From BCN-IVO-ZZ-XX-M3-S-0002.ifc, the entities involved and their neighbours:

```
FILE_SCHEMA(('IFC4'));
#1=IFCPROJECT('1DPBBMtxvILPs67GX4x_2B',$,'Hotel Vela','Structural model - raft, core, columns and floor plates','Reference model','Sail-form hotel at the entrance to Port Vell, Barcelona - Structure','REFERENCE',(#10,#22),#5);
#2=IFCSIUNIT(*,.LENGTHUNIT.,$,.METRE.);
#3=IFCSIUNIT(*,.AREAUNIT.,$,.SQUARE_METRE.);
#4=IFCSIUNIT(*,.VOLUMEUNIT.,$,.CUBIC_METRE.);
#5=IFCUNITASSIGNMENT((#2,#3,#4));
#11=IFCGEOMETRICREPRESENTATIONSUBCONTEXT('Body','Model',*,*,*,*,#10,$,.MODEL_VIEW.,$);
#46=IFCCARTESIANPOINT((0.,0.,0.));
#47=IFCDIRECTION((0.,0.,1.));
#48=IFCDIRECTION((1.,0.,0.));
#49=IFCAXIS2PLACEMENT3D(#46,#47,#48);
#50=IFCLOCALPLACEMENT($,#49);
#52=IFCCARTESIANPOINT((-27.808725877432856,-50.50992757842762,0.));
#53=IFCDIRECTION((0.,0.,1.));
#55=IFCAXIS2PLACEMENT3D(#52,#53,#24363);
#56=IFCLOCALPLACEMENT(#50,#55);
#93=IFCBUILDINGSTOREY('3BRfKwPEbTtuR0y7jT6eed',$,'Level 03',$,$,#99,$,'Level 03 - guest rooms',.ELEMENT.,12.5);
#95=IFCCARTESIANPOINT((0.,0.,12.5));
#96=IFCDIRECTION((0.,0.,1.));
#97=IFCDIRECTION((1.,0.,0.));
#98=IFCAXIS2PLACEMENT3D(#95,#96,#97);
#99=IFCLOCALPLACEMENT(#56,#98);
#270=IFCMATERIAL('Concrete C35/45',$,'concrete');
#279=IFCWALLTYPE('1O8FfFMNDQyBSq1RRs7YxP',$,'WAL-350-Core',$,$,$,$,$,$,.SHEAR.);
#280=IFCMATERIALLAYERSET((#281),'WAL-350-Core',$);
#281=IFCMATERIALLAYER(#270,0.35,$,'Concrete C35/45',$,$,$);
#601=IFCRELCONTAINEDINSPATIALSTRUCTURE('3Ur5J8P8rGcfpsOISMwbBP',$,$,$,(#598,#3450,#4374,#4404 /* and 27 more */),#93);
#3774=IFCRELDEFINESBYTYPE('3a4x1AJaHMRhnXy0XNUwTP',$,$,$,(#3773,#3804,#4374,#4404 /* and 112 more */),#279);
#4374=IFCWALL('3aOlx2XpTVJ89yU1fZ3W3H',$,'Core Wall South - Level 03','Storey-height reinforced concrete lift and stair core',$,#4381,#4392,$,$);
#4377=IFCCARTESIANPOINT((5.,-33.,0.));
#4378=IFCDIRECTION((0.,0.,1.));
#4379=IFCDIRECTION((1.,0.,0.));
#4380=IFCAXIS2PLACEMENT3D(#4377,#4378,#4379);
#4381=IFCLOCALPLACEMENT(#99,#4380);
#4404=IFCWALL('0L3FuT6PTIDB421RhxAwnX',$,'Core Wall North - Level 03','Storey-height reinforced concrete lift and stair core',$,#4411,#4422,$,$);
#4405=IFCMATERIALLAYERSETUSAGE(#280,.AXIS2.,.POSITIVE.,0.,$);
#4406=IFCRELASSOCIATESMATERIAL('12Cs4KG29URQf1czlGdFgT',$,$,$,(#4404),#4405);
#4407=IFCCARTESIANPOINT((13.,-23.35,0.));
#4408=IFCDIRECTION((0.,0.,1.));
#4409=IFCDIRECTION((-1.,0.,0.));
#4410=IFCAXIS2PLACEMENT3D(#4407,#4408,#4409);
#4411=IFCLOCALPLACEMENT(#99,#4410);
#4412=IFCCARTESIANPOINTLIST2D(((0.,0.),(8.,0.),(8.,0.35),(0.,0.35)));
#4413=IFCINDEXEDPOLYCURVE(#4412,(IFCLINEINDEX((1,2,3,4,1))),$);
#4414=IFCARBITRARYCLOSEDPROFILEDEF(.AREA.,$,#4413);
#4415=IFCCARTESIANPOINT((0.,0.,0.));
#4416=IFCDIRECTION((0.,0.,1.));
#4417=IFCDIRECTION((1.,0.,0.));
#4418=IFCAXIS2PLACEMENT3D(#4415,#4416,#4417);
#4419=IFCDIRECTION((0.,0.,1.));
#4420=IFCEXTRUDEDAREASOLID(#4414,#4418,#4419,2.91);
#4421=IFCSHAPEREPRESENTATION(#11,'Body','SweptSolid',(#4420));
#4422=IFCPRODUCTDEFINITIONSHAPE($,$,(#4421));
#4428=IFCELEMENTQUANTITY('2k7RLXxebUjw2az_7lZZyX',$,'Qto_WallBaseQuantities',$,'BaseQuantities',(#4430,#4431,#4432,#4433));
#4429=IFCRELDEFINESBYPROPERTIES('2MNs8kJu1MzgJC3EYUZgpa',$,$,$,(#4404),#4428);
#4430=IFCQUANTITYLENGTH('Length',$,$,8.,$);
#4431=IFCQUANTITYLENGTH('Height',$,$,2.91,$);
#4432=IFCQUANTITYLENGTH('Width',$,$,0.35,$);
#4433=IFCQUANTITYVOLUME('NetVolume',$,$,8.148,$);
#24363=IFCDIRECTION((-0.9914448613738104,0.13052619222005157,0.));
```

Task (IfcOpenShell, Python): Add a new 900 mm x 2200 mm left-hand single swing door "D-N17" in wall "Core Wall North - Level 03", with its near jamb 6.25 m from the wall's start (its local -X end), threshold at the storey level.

```python
import numpy as np
import ifcopenshell
import ifcopenshell.api.feature
import ifcopenshell.api.geometry
import ifcopenshell.api.pset
import ifcopenshell.api.root
import ifcopenshell.api.spatial
import ifcopenshell.geom
import ifcopenshell.util.element
import ifcopenshell.util.placement
import ifcopenshell.util.representation
import ifcopenshell.util.shape
import ifcopenshell.util.unit

model = ifcopenshell.open("BCN-IVO-ZZ-XX-M3-S-0002.ifc")
unit_scale = ifcopenshell.util.unit.calculate_unit_scale(model)
volume_scale = ifcopenshell.util.unit.calculate_unit_scale(model, "VOLUMEUNIT")
settings = ifcopenshell.geom.settings()


def volume(element):
    """Net volume in cubic metres, openings subtracted."""
    shape = ifcopenshell.geom.create_shape(settings, element)
    return ifcopenshell.util.shape.get_volume(shape.geometry)


wall = model.by_id(4404)
storey = ifcopenshell.util.element.get_container(wall, ifc_class="IfcBuildingStorey")
context = ifcopenshell.util.representation.get_context(model, "Model", "Body", "MODEL_VIEW")
before = volume(wall)

width, height, from_end, sill = 0.9, 2.2, 6.25, 0.0  # metres

# The wall runs along its own X axis, and the end named is its -X end.
wall_shape = ifcopenshell.geom.create_shape(settings, wall)
x, y, z = ifcopenshell.util.shape.get_vertices(wall_shape.geometry).T
start = x.min() + from_end
face, thickness = float(y.min()), float(y.max() - y.min())
wall_matrix = ifcopenshell.util.placement.get_local_placement(wall.ObjectPlacement)
level = ifcopenshell.util.placement.get_local_placement(storey.ObjectPlacement)[2, 3]


def in_wall(x, y):
    """Placement at x, y metres in the wall's axes, at sill height."""
    matrix = wall_matrix.copy()
    matrix[:, 3] = wall_matrix @ np.array([x / unit_scale, y / unit_scale, 0.0, 1.0])
    matrix[2, 3] = level + sill / unit_scale
    return matrix


# Opening: a box that overshoots both wall faces by 50 mm.
opening = ifcopenshell.api.root.create_entity(model, ifc_class="IfcOpeningElement", predefined_type="OPENING")
box = ifcopenshell.api.geometry.add_wall_representation(
    model, context=context, length=width, height=height, thickness=thickness + 0.1
)
ifcopenshell.api.geometry.assign_representation(model, product=opening, representation=box)
ifcopenshell.api.geometry.edit_object_placement(model, product=opening, matrix=in_wall(start, face - 0.05), is_si=False)
ifcopenshell.api.feature.add_feature(model, feature=opening, element=wall)

door = ifcopenshell.api.root.create_entity(model, ifc_class="IfcDoor", name="D-N17", predefined_type="DOOR")
door.OverallWidth, door.OverallHeight = width / unit_scale, height / unit_scale
door.OperationType = "SINGLE_SWING_LEFT"
body = ifcopenshell.api.geometry.add_door_representation(
    model,
    context=context,
    overall_width=door.OverallWidth,
    overall_height=door.OverallHeight,
    operation_type="SINGLE_SWING_LEFT",
    lining_properties={"LiningDepth": thickness / unit_scale, "ThresholdDepth": thickness / unit_scale},
)
ifcopenshell.api.geometry.assign_representation(model, product=door, representation=body)
ifcopenshell.api.spatial.assign_container(model, products=[door], relating_structure=storey)
ifcopenshell.api.feature.add_filling(model, opening=opening, element=door)

# The lining spans the wall, so the door starts at the wall face.
ifcopenshell.api.geometry.edit_object_placement(model, product=door, matrix=in_wall(start, face), is_si=False)

after = volume(wall)

# Update the wall's stored quantities.
qto = model.by_id(ifcopenshell.util.element.get_pset(wall, "Qto_WallBaseQuantities", should_inherit=False)["id"])
ifcopenshell.api.pset.edit_qto(model, qto=qto, properties={"NetVolume": after / volume_scale})

print(f"wall volume {before:.3f} -> {after:.3f} m3")

model.write("BCN-IVO-ZZ-XX-M3-S-0002_rev.ifc")
```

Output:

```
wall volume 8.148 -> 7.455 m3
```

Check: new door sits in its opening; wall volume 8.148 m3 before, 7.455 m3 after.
